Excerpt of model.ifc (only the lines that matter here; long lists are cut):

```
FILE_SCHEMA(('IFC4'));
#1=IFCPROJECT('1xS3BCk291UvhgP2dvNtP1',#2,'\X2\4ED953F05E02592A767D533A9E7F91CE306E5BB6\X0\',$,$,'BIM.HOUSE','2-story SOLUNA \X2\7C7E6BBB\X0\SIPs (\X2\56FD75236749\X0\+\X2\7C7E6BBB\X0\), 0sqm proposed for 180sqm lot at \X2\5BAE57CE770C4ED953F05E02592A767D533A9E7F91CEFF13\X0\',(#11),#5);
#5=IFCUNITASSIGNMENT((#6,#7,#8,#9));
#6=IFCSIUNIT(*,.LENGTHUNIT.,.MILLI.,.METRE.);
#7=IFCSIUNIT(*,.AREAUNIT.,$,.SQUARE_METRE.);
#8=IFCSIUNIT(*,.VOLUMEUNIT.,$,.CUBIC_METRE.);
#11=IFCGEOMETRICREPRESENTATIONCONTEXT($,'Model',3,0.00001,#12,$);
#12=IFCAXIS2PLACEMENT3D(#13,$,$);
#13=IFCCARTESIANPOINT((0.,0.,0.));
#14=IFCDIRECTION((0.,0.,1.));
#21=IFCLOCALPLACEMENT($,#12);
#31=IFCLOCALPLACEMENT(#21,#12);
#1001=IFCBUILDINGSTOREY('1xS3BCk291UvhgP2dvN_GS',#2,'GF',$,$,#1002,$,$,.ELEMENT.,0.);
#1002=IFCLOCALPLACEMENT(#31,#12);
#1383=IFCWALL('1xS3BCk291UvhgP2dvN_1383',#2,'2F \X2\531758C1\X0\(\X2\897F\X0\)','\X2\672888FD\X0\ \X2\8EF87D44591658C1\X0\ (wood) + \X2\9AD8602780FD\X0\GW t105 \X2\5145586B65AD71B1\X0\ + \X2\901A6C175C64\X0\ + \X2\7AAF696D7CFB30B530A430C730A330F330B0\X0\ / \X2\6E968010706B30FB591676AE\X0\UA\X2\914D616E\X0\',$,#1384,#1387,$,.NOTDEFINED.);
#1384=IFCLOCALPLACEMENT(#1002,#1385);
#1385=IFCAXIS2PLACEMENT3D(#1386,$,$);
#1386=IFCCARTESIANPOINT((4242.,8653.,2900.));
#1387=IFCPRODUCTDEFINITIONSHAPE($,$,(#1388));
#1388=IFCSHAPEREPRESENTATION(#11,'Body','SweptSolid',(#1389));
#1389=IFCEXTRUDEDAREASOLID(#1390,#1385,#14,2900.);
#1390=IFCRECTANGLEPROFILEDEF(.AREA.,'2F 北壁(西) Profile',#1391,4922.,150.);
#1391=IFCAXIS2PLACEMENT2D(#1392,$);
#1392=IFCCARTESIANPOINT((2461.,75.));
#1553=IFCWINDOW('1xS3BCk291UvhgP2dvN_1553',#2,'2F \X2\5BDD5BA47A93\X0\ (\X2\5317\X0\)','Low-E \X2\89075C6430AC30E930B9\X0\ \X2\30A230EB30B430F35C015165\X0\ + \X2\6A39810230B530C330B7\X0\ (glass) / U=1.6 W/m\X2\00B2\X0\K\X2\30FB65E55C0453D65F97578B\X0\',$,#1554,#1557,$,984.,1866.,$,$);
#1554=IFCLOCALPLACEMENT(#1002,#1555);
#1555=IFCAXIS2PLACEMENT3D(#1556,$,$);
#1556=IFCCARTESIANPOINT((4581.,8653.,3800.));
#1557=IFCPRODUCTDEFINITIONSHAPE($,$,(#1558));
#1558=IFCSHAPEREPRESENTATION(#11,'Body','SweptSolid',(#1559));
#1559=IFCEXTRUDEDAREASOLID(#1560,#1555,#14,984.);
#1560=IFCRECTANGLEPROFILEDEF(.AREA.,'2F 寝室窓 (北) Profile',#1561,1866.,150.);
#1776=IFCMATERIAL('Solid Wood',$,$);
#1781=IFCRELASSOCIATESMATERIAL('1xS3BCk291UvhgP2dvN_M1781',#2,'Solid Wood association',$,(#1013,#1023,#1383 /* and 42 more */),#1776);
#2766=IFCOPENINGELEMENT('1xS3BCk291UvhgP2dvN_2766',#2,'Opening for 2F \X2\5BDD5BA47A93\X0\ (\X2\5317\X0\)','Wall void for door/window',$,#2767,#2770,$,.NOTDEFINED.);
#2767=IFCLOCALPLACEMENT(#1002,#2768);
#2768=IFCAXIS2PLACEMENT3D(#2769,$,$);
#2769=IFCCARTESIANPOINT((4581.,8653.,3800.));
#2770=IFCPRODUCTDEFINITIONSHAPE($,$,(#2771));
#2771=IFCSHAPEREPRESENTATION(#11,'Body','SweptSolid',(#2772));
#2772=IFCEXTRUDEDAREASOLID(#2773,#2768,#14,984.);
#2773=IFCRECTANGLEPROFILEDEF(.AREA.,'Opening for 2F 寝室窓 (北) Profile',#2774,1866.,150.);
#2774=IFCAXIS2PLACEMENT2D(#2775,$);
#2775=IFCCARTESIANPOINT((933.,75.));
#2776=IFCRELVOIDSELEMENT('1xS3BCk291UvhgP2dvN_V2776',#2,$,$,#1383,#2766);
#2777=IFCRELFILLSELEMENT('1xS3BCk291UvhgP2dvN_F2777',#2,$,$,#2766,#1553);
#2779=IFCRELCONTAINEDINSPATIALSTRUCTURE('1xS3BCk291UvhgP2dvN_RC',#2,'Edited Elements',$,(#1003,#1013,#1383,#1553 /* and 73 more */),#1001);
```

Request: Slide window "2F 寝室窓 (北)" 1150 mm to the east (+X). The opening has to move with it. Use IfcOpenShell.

```python
import ifcopenshell
import ifcopenshell.api.geometry
import ifcopenshell.util.placement

model = ifcopenshell.open("model.ifc")

window = model.by_guid("1xS3BCk291UvhgP2dvN_1553")
opening = window.FillsVoids[0].RelatingOpeningElement
wall = opening.VoidsElements[0].RelatingBuildingElement

wall_matrix = ifcopenshell.util.placement.get_local_placement(wall.ObjectPlacement)
shift = wall_matrix[:3, 0] * 1150.0
before = ifcopenshell.util.placement.get_local_placement(window.ObjectPlacement)[:3, 3].copy()

# The window is not placed relative to its opening, so move both.
for product in (opening, window):
    matrix = ifcopenshell.util.placement.get_local_placement(product.ObjectPlacement)
    matrix[:3, 3] += shift
    ifcopenshell.api.geometry.edit_object_placement(model, product=product, matrix=matrix, is_si=False)

after = ifcopenshell.util.placement.get_local_placement(window.ObjectPlacement)[:3, 3]
print("window moved by", (after - before).round(3) + 0.0)

model.write("model_updated.ifc")
```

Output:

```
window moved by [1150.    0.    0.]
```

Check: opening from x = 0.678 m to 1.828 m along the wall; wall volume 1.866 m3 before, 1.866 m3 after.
